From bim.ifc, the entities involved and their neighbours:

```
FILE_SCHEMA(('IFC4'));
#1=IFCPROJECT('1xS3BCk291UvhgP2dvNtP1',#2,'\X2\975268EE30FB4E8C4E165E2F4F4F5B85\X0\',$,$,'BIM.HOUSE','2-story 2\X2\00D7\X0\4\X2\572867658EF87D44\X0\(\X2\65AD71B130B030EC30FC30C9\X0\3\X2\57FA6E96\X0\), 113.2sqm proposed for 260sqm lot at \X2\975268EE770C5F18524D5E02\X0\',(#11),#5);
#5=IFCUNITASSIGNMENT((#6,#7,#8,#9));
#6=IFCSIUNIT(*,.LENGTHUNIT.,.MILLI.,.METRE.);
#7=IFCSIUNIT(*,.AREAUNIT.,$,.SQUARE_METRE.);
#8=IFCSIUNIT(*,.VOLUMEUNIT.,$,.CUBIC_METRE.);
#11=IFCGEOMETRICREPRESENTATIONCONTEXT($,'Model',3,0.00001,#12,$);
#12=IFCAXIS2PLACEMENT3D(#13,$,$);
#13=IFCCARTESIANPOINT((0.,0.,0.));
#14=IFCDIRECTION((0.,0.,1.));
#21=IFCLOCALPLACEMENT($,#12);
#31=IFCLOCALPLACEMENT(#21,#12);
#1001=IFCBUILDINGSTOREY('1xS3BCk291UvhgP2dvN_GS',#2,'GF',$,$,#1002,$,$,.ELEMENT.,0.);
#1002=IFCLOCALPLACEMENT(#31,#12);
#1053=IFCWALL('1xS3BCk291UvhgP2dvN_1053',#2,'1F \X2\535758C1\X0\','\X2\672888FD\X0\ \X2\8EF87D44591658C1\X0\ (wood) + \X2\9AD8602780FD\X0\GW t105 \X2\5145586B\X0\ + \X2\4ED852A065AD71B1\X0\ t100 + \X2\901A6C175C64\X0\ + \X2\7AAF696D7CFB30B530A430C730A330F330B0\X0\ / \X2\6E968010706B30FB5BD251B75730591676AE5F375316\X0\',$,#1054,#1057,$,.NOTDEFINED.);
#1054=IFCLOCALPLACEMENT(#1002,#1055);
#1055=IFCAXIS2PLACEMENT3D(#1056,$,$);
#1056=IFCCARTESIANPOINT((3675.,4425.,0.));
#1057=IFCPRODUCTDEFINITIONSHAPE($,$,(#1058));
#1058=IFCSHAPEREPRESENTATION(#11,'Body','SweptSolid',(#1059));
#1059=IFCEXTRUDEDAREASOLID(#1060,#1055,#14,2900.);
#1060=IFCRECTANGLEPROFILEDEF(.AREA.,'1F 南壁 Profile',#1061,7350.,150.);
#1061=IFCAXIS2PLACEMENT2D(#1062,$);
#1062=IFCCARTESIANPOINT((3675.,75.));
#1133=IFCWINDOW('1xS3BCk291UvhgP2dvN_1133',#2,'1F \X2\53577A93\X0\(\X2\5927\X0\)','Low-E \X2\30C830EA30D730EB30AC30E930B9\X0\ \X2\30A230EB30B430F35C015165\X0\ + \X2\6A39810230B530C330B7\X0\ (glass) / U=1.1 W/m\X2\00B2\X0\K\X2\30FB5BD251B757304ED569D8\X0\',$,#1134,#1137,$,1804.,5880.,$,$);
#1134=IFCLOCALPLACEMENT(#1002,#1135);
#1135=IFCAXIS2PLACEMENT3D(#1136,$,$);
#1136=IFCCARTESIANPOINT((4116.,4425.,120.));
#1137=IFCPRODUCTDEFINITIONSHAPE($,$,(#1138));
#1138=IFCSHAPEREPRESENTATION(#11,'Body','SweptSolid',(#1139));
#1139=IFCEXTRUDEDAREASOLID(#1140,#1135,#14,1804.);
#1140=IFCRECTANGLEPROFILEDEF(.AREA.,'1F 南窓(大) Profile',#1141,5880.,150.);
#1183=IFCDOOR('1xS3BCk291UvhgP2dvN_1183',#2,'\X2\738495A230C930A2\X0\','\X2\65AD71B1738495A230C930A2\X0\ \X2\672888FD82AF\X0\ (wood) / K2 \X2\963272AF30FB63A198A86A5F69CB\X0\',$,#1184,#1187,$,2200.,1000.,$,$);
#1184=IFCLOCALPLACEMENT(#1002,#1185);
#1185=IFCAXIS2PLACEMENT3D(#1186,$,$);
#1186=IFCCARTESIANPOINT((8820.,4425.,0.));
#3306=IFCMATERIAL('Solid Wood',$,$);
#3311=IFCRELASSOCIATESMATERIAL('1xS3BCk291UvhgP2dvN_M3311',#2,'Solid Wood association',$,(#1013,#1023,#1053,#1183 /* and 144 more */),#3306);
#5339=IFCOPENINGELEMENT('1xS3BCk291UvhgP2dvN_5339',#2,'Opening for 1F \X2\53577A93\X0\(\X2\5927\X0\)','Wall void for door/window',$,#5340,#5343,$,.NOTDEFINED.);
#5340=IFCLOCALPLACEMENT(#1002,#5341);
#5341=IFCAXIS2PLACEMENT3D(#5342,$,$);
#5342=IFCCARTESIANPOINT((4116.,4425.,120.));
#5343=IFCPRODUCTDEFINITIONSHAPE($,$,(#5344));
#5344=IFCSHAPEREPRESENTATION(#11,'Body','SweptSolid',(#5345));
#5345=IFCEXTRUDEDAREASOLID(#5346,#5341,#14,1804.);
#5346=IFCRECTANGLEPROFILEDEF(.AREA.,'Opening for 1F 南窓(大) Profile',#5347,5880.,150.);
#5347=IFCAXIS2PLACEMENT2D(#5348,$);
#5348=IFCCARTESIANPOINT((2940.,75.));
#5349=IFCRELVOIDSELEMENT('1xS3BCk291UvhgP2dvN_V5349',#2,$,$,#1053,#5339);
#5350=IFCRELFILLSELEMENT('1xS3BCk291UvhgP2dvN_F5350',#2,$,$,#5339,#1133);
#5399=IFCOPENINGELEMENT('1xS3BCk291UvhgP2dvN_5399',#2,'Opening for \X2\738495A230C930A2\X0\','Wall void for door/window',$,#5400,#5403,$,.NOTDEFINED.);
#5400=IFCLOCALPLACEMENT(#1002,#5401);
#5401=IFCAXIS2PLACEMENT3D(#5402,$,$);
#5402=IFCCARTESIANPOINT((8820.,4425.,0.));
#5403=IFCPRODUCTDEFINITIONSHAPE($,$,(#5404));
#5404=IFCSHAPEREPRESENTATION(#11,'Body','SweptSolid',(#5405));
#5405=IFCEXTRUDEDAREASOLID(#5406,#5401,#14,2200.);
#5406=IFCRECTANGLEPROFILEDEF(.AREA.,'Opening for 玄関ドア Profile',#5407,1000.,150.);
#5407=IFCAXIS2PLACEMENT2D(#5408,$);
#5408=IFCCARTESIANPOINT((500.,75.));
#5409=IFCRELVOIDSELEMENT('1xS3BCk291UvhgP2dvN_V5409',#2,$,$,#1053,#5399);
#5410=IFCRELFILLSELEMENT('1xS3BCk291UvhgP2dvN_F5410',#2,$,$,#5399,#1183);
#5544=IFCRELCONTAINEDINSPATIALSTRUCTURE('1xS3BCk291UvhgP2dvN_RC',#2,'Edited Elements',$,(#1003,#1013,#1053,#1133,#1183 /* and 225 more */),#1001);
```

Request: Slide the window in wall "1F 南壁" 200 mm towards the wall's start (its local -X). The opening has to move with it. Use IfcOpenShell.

```python
import ifcopenshell
import ifcopenshell.api.geometry
import ifcopenshell.util.placement

model = ifcopenshell.open("bim.ifc")

window = model.by_guid("1xS3BCk291UvhgP2dvN_1133")
opening = window.FillsVoids[0].RelatingOpeningElement
wall = opening.VoidsElements[0].RelatingBuildingElement

wall_matrix = ifcopenshell.util.placement.get_local_placement(wall.ObjectPlacement)
shift = wall_matrix[:3, 0] * -200.0
before = ifcopenshell.util.placement.get_local_placement(window.ObjectPlacement)[:3, 3].copy()

# The window is not placed relative to its opening, so move both.
for product in (opening, window):
    matrix = ifcopenshell.util.placement.get_local_placement(product.ObjectPlacement)
    matrix[:3, 3] += shift
    ifcopenshell.api.geometry.edit_object_placement(model, product=product, matrix=matrix, is_si=False)

after = ifcopenshell.util.placement.get_local_placement(window.ObjectPlacement)[:3, 3]
print("window moved by", (after - before).round(3) + 0.0)

model.write("bim_v2.ifc")
```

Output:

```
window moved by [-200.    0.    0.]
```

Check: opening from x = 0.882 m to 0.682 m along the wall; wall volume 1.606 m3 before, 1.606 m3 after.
